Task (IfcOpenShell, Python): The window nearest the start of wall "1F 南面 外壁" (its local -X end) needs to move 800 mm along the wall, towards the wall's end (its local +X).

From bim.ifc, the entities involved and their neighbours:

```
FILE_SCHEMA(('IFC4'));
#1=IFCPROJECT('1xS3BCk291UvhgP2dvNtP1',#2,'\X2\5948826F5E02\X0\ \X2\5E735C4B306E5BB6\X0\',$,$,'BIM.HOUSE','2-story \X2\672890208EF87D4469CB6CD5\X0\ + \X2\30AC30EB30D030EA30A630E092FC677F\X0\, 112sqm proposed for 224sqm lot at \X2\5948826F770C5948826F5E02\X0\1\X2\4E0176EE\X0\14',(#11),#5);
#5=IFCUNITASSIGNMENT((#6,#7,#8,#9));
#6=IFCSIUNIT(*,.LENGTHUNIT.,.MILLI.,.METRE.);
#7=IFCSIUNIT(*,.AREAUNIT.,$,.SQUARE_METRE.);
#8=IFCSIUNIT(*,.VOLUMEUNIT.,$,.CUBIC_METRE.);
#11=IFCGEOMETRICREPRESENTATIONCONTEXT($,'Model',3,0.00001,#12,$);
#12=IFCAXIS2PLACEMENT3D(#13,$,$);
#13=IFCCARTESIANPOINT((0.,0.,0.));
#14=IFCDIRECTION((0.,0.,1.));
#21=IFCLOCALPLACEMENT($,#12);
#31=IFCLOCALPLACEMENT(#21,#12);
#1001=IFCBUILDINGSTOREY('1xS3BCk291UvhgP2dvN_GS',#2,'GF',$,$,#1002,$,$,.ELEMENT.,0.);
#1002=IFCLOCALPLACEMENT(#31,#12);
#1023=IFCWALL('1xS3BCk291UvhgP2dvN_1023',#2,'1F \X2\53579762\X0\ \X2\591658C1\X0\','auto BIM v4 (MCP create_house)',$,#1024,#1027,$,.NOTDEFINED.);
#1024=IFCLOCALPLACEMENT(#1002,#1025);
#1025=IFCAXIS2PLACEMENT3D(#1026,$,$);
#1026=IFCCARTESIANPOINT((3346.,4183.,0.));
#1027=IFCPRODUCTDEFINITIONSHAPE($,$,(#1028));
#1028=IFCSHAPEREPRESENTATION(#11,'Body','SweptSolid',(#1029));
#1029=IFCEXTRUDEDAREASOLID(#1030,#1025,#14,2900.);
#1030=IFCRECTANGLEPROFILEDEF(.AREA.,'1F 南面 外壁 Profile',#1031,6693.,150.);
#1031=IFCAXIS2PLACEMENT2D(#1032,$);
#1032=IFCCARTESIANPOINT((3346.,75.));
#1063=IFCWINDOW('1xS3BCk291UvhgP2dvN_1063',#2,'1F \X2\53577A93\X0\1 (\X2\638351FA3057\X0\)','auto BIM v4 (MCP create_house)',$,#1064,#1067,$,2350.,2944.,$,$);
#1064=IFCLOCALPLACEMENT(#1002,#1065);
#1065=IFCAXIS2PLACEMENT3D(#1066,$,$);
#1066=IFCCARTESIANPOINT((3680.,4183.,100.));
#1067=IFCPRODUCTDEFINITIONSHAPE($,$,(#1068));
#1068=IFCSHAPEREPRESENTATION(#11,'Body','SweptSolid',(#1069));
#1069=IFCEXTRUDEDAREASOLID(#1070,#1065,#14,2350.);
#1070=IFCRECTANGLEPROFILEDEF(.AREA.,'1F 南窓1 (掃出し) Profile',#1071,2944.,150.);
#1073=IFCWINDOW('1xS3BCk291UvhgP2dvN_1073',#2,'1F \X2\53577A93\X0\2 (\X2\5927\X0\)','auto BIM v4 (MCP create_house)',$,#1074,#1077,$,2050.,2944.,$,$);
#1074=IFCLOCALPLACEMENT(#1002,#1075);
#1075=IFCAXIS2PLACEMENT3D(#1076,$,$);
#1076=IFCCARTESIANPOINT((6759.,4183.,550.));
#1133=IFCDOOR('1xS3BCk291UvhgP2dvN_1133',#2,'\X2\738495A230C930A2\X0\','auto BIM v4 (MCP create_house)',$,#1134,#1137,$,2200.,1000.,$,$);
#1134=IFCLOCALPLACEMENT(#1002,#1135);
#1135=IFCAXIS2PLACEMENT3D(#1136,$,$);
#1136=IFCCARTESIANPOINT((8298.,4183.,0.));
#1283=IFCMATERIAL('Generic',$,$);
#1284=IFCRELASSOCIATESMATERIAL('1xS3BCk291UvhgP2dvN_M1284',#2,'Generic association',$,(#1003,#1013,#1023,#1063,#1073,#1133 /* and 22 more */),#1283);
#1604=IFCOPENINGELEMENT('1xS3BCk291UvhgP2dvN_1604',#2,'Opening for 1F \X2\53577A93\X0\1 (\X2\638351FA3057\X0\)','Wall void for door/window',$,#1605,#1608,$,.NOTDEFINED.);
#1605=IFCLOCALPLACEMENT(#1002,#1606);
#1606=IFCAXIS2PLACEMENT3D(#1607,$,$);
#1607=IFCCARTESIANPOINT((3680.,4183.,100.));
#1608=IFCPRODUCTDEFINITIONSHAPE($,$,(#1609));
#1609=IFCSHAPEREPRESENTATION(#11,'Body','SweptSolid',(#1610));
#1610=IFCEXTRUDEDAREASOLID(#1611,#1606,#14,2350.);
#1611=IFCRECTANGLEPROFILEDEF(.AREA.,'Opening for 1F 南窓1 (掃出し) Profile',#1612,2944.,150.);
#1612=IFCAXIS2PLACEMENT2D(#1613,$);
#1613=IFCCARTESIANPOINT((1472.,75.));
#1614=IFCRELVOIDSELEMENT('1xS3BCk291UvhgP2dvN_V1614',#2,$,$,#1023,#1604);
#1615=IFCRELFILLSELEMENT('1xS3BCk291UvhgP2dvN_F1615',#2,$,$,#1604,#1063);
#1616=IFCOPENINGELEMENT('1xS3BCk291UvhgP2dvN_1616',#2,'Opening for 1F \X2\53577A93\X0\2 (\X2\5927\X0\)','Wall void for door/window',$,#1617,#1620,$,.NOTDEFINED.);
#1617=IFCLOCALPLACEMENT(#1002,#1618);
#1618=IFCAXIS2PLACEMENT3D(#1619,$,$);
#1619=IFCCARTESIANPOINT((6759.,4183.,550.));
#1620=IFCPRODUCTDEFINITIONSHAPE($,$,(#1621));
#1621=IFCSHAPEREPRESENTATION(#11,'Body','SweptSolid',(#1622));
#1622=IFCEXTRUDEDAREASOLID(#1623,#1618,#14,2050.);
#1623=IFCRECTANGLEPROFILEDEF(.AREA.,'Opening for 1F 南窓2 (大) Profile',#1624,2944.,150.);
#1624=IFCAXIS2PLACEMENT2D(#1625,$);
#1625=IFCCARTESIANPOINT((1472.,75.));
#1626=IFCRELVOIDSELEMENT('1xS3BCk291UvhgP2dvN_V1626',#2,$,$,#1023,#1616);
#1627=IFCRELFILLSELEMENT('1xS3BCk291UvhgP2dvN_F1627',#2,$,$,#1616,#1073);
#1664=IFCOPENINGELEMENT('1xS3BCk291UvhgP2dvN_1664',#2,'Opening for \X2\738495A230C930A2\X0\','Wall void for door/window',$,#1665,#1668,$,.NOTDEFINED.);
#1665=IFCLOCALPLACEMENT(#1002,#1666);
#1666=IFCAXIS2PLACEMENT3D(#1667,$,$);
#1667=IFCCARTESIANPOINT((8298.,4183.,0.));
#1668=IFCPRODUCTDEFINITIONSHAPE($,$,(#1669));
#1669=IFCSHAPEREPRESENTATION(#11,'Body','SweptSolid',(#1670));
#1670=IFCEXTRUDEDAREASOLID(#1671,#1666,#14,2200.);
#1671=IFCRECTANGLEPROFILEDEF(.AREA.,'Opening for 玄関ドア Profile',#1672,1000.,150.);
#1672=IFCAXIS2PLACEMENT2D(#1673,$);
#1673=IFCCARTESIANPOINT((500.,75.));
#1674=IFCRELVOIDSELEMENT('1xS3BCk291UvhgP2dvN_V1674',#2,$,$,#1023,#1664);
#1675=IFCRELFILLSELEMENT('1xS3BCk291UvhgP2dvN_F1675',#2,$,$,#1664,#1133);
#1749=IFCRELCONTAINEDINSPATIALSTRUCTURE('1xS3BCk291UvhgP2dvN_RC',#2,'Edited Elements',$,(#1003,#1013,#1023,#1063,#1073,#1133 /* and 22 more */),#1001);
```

```python
import ifcopenshell
import ifcopenshell.api.geometry
import ifcopenshell.util.placement
import ifcopenshell.util.unit

model = ifcopenshell.open("bim.ifc")
unit_scale = ifcopenshell.util.unit.calculate_unit_scale(model)

window = model.by_id(1063)
opening = window.FillsVoids[0].RelatingOpeningElement
wall = opening.VoidsElements[0].RelatingBuildingElement

wall_matrix = ifcopenshell.util.placement.get_local_placement(wall.ObjectPlacement)
shift = wall_matrix[:3, 0] * 0.8 / unit_scale
before = ifcopenshell.util.placement.get_local_placement(window.ObjectPlacement)[:3, 3].copy()

# The window is not placed relative to its opening, so move both.
for product in (opening, window):
    matrix = ifcopenshell.util.placement.get_local_placement(product.ObjectPlacement)
    matrix[:3, 3] += shift
    ifcopenshell.api.geometry.edit_object_placement(model, product=product, matrix=matrix, is_si=False)

after = ifcopenshell.util.placement.get_local_placement(window.ObjectPlacement)[:3, 3]
print("window moved by", (after - before).round(3) + 0.0)

model.write("bim-out.ifc")
```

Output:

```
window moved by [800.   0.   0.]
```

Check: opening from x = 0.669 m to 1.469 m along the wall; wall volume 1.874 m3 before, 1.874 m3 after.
